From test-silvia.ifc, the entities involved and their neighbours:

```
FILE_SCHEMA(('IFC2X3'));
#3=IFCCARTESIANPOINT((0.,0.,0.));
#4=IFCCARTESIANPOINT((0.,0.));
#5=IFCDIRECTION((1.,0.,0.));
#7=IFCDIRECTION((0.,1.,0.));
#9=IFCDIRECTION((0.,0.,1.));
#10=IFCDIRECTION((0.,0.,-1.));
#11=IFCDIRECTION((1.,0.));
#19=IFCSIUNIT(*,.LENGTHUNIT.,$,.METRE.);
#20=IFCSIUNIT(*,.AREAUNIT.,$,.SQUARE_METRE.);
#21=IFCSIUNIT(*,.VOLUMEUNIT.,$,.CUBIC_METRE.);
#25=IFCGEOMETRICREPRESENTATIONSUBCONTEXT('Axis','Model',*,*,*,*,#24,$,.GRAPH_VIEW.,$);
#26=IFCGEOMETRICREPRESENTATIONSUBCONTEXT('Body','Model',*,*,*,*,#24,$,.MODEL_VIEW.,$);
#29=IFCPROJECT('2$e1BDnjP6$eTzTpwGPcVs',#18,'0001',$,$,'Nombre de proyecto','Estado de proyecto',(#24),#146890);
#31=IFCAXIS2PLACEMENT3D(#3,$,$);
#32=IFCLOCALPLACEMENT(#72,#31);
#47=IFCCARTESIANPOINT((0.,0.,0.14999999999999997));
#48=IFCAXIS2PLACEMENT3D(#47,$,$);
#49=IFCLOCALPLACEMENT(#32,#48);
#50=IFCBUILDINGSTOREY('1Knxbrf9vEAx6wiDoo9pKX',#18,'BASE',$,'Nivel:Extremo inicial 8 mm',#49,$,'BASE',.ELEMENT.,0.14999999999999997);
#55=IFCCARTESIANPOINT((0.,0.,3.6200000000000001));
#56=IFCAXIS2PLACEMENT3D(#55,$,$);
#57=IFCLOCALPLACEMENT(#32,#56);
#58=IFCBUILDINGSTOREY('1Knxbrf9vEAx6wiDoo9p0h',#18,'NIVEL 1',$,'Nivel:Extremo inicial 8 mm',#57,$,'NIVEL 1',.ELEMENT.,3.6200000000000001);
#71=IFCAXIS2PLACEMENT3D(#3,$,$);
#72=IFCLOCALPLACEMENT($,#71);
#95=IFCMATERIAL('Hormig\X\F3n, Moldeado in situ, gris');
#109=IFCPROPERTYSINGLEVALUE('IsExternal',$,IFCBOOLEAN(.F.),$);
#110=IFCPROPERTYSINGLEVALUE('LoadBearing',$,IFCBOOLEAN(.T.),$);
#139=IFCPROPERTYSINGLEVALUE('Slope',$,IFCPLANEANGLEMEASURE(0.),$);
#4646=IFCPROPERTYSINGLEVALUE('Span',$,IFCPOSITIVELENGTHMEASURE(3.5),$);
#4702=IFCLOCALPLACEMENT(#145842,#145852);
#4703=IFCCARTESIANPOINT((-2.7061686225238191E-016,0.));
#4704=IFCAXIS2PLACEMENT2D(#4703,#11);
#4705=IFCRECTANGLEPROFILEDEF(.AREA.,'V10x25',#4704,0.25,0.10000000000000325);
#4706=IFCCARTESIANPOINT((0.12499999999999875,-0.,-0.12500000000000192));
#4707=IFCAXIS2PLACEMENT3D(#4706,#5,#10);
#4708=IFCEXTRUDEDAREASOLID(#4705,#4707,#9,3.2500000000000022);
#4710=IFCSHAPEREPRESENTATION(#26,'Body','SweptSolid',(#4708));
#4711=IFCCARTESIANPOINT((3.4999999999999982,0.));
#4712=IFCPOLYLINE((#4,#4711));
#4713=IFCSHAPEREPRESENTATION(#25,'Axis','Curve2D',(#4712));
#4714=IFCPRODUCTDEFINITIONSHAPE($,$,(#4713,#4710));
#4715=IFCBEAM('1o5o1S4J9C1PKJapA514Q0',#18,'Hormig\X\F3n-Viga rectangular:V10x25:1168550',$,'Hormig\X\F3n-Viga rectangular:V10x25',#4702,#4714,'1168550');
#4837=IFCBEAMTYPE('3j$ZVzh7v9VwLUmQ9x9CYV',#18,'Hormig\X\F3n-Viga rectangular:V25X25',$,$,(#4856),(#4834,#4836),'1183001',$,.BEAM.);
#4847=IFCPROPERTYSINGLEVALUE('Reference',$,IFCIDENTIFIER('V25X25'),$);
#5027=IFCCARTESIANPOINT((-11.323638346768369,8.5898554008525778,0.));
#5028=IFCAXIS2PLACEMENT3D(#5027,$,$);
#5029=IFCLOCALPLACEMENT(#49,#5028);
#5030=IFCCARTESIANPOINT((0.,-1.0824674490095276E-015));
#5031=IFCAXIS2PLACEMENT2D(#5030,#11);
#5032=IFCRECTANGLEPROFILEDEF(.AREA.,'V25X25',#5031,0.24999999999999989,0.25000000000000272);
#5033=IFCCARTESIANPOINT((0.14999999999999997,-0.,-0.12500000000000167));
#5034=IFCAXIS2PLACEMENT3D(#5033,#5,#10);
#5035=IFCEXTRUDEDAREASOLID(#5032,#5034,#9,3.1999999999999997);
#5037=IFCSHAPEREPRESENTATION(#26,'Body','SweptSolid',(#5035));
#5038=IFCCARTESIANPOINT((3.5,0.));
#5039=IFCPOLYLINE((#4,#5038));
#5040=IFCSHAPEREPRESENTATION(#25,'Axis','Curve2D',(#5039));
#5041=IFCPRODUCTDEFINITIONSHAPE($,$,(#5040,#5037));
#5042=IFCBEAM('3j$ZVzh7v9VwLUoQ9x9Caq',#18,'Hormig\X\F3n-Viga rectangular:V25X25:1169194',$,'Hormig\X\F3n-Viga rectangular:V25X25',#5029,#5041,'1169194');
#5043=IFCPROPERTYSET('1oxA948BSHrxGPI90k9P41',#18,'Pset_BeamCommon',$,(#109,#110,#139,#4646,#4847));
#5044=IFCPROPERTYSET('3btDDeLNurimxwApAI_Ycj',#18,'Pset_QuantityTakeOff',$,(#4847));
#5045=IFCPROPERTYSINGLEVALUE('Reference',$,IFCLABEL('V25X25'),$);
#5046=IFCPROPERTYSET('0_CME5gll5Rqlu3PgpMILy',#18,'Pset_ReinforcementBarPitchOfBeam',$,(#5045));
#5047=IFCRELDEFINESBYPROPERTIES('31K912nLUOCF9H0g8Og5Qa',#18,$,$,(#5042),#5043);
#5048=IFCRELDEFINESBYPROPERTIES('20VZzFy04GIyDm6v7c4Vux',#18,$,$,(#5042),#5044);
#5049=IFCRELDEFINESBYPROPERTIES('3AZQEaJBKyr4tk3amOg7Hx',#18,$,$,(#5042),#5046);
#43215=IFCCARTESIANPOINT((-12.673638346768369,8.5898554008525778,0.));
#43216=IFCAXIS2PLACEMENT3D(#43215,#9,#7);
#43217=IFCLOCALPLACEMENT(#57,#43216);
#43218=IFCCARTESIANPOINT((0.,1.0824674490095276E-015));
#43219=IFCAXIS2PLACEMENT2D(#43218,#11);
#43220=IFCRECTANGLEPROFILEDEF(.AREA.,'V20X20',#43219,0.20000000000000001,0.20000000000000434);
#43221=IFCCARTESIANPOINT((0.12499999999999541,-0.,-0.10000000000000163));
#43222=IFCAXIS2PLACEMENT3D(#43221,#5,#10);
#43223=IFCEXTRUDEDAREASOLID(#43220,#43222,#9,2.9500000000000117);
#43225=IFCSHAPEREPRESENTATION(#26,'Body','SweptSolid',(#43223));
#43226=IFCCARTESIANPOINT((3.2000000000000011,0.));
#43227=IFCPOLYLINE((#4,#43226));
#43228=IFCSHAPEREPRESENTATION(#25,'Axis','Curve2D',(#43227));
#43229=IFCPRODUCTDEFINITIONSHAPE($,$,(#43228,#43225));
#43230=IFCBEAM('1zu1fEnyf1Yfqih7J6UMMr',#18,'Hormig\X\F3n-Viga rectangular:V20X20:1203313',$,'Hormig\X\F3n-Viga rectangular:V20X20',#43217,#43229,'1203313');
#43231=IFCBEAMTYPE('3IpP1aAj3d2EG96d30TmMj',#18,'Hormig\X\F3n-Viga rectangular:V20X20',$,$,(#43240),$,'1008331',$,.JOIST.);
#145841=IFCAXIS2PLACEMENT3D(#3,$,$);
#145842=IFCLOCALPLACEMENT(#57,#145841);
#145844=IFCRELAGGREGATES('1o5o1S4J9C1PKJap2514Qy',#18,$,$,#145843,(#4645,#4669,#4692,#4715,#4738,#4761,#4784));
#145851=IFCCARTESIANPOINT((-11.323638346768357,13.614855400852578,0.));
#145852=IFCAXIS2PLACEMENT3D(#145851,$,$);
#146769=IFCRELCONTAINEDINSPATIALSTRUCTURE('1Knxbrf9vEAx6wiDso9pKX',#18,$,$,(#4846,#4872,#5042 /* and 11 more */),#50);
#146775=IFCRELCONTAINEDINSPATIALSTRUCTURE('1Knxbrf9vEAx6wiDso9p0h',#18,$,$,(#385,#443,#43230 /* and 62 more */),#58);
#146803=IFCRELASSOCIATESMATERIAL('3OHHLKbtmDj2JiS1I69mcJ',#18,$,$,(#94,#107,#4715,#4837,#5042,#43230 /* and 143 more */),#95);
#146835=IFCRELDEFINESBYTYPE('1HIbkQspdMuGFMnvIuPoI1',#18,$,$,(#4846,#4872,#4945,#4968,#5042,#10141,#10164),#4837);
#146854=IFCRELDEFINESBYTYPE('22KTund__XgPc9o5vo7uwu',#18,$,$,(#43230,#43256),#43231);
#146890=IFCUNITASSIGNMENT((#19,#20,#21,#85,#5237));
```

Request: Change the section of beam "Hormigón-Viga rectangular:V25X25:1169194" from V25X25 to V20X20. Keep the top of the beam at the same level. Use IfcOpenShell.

```python
import ifcopenshell
import ifcopenshell.api.pset
import ifcopenshell.api.type
import ifcopenshell.util.element
import ifcopenshell.util.representation

model = ifcopenshell.open("test-silvia.ifc")

member = model.by_id(5042)
source = next(p for p in model.by_type("IfcRectangleProfileDef") if p.ProfileName == "V20X20")

body = ifcopenshell.util.representation.get_representation(member, "Model", "Body")
solid = body.Items[0]
old_profile = solid.SweptArea

# Copy the section's sizes but keep this member's own profile position.
profile = ifcopenshell.util.element.copy(model, source)
# Profiles are centred, so shift by half the change in depth to hold the top.
shift = (old_profile.XDim - profile.XDim) / 2
x, y = old_profile.Position.Location.Coordinates
up = (-1.0, 0.0)  # upwards, in the solid's own plane
location = model.createIfcCartesianPoint((x + up[0] * shift, y + up[1] * shift))
profile.Position = model.createIfcAxis2Placement2D(location, old_profile.Position.RefDirection)
solid.SweptArea = profile
if not model.get_total_inverses(old_profile):
    ifcopenshell.util.element.remove_deep2(model, old_profile)

new_type = model.by_guid("3IpP1aAj3d2EG96d30TmMj")
ifcopenshell.api.type.assign_type(
    model, related_objects=[member], relating_type=new_type, should_map_representations=False
)
member.Name = member.Name.replace("V25X25", "V20X20")
member.ObjectType = "Hormigón-Viga rectangular:V20X20"
pset = model.by_id(ifcopenshell.util.element.get_pset(member, "Pset_BeamCommon", should_inherit=False)["id"])
ifcopenshell.api.pset.edit_pset(model, pset=pset, properties={"Reference": "V20X20"})
pset = model.by_id(ifcopenshell.util.element.get_pset(member, "Pset_QuantityTakeOff", should_inherit=False)["id"])
ifcopenshell.api.pset.edit_pset(model, pset=pset, properties={"Reference": "V20X20"})
pset = model.by_id(ifcopenshell.util.element.get_pset(member, "Pset_ReinforcementBarPitchOfBeam", should_inherit=False)["id"])
ifcopenshell.api.pset.edit_pset(model, pset=pset, properties={"Reference": "V20X20"})

print(solid.SweptArea)

model.write("test-silvia-out.ifc")
```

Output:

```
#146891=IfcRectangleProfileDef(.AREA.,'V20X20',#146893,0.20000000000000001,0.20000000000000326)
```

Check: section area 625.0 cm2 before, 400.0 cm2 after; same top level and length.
